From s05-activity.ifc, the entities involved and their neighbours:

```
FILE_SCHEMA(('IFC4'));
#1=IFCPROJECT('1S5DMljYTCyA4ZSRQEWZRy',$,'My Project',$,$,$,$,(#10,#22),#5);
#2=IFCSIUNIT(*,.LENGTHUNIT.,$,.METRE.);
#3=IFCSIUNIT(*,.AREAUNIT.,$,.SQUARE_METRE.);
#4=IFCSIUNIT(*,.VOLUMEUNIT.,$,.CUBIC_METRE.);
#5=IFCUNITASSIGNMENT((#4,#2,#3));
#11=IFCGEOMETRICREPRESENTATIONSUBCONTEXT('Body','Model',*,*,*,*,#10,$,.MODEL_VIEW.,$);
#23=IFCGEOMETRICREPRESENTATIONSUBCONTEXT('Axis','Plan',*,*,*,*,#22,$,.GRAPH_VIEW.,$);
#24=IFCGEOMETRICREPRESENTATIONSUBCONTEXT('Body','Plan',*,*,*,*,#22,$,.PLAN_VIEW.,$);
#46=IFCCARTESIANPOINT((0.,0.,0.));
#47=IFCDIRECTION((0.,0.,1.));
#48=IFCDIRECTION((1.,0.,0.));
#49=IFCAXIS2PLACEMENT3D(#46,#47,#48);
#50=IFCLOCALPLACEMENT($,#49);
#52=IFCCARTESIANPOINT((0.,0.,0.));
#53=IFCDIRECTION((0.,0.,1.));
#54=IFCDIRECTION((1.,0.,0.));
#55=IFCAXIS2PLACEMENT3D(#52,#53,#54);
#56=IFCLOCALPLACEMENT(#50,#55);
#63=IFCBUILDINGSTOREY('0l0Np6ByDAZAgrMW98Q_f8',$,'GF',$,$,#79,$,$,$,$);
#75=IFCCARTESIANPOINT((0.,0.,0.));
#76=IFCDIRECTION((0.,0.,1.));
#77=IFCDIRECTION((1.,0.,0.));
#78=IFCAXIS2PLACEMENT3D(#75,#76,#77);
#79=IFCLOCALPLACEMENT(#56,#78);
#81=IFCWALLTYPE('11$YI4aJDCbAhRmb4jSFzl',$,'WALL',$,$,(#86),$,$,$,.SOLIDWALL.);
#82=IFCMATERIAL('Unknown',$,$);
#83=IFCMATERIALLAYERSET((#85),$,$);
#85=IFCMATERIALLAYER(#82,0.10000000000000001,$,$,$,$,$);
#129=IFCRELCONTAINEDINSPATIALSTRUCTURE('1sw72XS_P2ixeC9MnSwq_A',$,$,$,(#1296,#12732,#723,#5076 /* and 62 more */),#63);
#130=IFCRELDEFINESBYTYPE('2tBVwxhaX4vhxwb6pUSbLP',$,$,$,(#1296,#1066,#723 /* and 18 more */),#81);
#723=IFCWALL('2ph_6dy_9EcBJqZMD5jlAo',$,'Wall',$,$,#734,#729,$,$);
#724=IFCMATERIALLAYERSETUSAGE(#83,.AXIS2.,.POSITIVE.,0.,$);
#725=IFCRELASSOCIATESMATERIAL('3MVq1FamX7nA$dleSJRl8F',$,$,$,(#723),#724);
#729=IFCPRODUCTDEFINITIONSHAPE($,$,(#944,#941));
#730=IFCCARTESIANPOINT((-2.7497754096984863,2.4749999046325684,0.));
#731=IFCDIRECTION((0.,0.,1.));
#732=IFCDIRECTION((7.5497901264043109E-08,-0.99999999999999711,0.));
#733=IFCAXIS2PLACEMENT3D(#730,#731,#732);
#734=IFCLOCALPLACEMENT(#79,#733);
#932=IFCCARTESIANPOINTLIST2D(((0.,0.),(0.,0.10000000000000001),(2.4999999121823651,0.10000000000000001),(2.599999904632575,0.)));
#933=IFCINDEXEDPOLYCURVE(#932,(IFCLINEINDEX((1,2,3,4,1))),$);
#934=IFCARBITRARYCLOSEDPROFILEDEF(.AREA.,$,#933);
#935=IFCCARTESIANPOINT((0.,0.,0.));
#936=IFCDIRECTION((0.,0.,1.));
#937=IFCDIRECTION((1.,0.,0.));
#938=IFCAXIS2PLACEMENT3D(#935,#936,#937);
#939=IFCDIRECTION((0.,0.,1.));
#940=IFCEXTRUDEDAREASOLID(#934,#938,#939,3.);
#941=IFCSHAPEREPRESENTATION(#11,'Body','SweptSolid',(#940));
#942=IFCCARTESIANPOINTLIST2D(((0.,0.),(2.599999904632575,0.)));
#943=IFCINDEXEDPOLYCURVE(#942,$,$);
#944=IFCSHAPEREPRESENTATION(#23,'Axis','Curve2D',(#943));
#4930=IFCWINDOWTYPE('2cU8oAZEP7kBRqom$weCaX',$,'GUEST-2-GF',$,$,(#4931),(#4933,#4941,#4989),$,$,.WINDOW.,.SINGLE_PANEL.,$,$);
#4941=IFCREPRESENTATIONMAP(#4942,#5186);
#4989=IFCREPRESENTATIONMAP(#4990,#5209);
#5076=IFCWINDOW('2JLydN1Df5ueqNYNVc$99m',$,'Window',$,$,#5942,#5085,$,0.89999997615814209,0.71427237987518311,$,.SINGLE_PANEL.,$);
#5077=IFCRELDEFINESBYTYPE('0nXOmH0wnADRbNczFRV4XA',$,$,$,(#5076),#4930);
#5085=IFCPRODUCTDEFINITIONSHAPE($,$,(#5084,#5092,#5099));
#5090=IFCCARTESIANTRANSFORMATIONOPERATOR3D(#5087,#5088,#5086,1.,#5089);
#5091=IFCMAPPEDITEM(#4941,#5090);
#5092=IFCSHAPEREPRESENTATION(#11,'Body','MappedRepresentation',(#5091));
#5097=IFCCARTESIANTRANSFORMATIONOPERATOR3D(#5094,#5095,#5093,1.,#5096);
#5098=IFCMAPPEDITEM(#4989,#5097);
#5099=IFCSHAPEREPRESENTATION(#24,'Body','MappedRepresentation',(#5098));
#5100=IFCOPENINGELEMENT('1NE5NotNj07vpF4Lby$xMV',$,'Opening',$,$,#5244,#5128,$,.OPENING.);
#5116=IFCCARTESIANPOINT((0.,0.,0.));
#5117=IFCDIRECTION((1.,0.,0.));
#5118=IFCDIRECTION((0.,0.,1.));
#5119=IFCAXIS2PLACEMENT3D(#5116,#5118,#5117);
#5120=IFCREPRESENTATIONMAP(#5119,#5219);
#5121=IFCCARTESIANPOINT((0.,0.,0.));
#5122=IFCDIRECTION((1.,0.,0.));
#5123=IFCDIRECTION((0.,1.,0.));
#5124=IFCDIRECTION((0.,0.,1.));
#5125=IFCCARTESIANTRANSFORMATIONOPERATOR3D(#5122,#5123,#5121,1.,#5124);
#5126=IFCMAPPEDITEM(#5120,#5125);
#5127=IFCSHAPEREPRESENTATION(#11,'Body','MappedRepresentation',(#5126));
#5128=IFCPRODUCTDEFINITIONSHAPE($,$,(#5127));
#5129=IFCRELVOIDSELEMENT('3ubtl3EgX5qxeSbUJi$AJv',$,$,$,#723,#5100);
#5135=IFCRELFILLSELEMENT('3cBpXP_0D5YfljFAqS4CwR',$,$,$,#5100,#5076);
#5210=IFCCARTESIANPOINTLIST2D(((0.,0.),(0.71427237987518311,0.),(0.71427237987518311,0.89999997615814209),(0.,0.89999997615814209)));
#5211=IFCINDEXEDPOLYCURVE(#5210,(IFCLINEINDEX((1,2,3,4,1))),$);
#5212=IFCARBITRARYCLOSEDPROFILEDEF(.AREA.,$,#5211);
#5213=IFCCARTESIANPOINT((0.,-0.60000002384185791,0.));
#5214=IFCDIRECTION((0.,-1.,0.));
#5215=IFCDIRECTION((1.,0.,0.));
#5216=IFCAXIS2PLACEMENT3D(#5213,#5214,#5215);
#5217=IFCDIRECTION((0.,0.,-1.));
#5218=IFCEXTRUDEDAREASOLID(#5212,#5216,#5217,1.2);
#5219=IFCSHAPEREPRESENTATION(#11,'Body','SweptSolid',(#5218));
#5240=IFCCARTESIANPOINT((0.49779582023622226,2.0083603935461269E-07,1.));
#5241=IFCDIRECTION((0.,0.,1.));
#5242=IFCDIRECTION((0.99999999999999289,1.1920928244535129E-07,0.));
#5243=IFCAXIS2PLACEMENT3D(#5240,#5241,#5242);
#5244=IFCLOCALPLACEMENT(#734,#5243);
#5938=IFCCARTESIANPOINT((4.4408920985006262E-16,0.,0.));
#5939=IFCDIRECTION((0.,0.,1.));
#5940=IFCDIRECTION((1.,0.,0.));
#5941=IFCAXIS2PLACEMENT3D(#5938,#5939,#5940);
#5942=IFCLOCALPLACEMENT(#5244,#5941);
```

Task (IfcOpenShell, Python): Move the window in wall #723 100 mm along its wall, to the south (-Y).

```python
import ifcopenshell
import ifcopenshell.api.geometry
import ifcopenshell.util.placement
import ifcopenshell.util.unit

model = ifcopenshell.open("s05-activity.ifc")
unit_scale = ifcopenshell.util.unit.calculate_unit_scale(model)

window = model.by_id(5076)
opening = window.FillsVoids[0].RelatingOpeningElement
wall = opening.VoidsElements[0].RelatingBuildingElement

wall_matrix = ifcopenshell.util.placement.get_local_placement(wall.ObjectPlacement)
shift = wall_matrix[:3, 0] * 0.1 / unit_scale
before = ifcopenshell.util.placement.get_local_placement(window.ObjectPlacement)[:3, 3].copy()

# The window is placed relative to its opening, so it follows when the opening moves.
matrix = ifcopenshell.util.placement.get_local_placement(opening.ObjectPlacement)
matrix[:3, 3] += shift
ifcopenshell.api.geometry.edit_object_placement(
    model, product=opening, matrix=matrix, is_si=False, should_transform_children=True
)

after = ifcopenshell.util.placement.get_local_placement(window.ObjectPlacement)[:3, 3]
print("window moved by", (after - before).round(3) + 0.0)

model.write("s05-activity_v2.ifc")
```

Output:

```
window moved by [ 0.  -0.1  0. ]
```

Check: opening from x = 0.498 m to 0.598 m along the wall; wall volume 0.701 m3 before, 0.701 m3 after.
